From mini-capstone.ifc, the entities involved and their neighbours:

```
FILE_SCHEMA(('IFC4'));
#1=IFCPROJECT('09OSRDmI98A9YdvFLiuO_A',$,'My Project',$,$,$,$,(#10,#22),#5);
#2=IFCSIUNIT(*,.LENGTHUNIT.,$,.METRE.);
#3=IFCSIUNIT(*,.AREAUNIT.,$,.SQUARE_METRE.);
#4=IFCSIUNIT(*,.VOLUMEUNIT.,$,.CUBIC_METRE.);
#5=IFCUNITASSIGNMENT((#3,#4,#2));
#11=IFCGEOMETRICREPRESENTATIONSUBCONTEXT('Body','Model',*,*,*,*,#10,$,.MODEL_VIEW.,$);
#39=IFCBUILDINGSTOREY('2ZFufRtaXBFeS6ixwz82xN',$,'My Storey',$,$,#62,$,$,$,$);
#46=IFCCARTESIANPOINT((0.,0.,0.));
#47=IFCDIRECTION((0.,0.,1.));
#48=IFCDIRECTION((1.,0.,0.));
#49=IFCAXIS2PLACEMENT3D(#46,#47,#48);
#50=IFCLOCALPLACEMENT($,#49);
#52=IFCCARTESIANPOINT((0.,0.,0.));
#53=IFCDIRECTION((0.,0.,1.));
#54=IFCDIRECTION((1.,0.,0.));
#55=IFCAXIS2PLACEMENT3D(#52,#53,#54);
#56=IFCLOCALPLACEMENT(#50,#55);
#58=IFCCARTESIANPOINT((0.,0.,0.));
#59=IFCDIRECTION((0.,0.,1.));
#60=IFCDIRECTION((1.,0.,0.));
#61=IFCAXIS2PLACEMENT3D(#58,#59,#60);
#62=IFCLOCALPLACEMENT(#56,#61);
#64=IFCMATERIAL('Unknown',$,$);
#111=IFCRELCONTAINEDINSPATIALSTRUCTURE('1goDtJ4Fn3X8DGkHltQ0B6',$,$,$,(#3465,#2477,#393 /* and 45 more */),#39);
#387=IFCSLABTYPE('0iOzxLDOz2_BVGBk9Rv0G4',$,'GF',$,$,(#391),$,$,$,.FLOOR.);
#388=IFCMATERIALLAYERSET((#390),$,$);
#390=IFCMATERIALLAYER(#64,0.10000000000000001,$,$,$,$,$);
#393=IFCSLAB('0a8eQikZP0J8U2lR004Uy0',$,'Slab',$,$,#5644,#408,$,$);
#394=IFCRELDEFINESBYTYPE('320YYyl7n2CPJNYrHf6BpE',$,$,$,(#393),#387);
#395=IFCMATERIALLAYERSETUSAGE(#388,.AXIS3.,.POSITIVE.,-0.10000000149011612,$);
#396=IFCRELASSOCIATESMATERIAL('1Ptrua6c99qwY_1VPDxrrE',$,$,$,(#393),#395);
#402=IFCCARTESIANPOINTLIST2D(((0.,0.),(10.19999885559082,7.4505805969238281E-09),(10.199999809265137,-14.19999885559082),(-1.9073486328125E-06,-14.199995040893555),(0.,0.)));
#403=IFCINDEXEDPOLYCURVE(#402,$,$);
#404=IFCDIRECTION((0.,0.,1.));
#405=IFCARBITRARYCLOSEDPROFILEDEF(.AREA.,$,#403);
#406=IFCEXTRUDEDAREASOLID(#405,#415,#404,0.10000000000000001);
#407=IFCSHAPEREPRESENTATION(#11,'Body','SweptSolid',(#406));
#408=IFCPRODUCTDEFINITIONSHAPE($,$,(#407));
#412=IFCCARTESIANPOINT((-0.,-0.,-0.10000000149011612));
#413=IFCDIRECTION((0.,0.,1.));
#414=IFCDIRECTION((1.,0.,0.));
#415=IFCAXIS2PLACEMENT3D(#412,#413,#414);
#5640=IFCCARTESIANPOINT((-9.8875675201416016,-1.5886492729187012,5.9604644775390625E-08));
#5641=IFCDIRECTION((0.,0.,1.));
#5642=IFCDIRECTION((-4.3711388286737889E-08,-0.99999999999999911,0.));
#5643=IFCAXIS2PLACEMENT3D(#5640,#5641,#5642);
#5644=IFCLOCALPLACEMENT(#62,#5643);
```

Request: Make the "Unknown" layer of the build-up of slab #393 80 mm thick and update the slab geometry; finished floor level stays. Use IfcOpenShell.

```python
import ifcopenshell
import ifcopenshell.util.element
import ifcopenshell.util.representation
import ifcopenshell.util.unit

model = ifcopenshell.open("mini-capstone.ifc")
unit_scale = ifcopenshell.util.unit.calculate_unit_scale(model)

layer_set = model.by_id(388)
layer = next(l for l in layer_set.MaterialLayers if l.Material and l.Material.Name == "Unknown")
change = 0.08 / unit_scale - layer.LayerThickness
layer.LayerThickness += change

# Geometry does not follow the layer set by itself.
slabs = [e for e in ifcopenshell.util.element.get_elements_by_material(model, layer_set) if e.is_a("IfcSlab")]
for slab in sorted(slabs, key=lambda e: e.id()):
    body = ifcopenshell.util.representation.get_representation(slab, "Model", "Body")
    solid = body.Items[0]
    old_depth = solid.Depth
    solid.Depth += change
    # Extruded upwards: lower the start of the extrusion so the top stays.
    x, y, z = solid.Position.Location.Coordinates
    solid.Position.Location = model.createIfcCartesianPoint((x, y, z - change))
    print(slab.id(), f"{old_depth:g} -> {solid.Depth:g}")

# The layers are counted up from the underside, which has moved.
for usage in {ifcopenshell.util.element.get_material(slab) for slab in slabs}:
    usage.OffsetFromReferenceLine -= change

model.write("mini-capstone_edited.ifc")
```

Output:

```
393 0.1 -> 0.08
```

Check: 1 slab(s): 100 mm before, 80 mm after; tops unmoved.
